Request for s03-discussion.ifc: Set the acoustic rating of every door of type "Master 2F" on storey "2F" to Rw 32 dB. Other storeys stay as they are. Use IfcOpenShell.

First a look at what the model holds.

```python
import ifcopenshell
import ifcopenshell.util.element

model = ifcopenshell.open("s03-discussion.ifc")
print(model.schema)
storey = next(s for s in model.by_type("IfcBuildingStorey") if s.Name == "2F")
doors = [e for e in ifcopenshell.util.element.get_decomposition(storey) if e.is_a("IfcDoor")]
seen = {}
for e in doors:
    element_type = ifcopenshell.util.element.get_type(e)
    key = (element_type.Name if element_type != e and element_type else None, ifcopenshell.util.element.get_pset(e, "Pset_DoorCommon", "AcousticRating"))
    seen[key] = seen.get(key, 0) + 1
for (name, value), count in sorted(seen.items(), key=str):
    print(count, "x", name, "|", value)
```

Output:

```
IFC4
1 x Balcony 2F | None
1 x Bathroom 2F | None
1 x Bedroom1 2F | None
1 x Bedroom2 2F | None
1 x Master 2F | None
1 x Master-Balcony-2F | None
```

```python
import ifcopenshell
import ifcopenshell.api.pset
import ifcopenshell.util.element

model = ifcopenshell.open("s03-discussion.ifc")

storey = next(s for s in model.by_type("IfcBuildingStorey") if s.Name == "2F")
doors = [e for e in ifcopenshell.util.element.get_decomposition(storey) if e.is_a("IfcDoor")]

count = 0
for e in doors:
    element_type = ifcopenshell.util.element.get_type(e)
    if element_type in (None, e) or element_type.Name != "Master 2F":
        continue
    # add_pset returns the element's existing set when there is one.
    pset = ifcopenshell.api.pset.add_pset(model, product=e, name="Pset_DoorCommon")
    ifcopenshell.api.pset.edit_pset(model, pset=pset, properties={"AcousticRating": "Rw 32 dB"})
    count += 1

print(count, "doors updated")

model.write("s03-discussion-out.ifc")
```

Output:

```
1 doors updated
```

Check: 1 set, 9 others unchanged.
